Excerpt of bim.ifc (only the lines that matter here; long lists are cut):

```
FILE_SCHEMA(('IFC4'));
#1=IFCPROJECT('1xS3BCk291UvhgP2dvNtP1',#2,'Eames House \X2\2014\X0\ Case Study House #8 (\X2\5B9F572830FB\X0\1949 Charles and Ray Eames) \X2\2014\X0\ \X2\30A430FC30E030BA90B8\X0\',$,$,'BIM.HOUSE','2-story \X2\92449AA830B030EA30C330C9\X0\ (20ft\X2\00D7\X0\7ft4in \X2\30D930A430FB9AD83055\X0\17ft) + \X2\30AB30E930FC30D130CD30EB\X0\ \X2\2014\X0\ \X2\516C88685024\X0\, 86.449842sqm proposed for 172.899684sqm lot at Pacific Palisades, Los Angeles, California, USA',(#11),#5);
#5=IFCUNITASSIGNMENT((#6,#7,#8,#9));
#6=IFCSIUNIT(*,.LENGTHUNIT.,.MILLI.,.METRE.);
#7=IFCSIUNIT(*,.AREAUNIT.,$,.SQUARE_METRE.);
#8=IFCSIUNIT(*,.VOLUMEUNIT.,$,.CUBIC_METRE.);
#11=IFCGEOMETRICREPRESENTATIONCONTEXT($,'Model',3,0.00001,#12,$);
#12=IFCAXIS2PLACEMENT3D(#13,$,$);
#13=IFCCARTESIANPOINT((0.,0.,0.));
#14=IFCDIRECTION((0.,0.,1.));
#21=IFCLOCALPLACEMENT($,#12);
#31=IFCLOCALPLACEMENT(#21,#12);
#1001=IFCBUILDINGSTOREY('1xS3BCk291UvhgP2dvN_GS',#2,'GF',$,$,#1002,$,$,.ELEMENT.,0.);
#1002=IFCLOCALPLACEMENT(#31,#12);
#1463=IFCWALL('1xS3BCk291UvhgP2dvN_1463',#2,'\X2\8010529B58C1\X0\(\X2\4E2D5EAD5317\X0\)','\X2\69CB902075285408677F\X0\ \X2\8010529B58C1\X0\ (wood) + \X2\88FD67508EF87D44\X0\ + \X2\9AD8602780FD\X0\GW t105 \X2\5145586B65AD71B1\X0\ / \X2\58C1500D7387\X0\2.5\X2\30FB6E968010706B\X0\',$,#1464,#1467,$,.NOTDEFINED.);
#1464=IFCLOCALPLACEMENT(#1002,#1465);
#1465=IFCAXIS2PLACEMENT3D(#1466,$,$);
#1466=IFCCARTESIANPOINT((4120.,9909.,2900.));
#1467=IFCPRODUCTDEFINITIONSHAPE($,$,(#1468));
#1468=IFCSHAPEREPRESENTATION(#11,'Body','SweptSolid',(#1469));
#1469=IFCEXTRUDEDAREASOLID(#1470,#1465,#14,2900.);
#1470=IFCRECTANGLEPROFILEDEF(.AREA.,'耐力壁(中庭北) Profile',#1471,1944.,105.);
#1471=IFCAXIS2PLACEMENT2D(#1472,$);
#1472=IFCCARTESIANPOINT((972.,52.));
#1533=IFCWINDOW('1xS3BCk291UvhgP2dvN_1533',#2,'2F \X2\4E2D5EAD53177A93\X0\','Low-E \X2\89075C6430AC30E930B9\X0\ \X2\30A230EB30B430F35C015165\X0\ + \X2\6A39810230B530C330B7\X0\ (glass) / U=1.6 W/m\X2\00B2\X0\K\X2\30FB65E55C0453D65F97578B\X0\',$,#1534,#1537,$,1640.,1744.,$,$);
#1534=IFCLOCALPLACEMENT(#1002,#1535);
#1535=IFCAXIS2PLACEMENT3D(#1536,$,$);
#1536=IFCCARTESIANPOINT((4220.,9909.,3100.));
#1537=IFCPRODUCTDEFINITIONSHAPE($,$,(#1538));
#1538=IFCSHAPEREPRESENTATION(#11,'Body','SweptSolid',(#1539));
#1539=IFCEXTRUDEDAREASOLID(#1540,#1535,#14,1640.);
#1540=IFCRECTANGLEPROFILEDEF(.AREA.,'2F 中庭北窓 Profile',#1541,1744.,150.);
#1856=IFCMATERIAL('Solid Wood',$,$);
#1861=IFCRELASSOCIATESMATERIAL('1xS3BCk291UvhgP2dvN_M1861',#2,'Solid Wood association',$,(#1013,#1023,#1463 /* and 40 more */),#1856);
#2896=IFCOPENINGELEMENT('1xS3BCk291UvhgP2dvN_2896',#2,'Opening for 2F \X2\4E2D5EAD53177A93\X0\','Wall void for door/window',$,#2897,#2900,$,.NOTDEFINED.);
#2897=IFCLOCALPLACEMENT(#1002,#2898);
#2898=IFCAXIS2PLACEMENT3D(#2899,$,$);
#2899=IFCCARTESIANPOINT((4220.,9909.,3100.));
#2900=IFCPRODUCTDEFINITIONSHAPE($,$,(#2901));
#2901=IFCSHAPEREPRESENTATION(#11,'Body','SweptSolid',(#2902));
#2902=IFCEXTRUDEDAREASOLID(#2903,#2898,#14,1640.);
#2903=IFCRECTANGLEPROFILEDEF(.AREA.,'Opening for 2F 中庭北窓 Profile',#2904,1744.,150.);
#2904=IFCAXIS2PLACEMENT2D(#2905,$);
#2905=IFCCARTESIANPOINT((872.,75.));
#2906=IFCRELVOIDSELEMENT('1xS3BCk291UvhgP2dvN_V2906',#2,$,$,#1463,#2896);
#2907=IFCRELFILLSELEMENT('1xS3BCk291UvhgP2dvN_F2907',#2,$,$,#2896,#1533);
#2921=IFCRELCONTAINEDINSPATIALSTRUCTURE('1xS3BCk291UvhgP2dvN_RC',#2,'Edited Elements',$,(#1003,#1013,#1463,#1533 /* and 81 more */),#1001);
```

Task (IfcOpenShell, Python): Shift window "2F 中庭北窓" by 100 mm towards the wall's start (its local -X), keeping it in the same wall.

```python
import ifcopenshell
import ifcopenshell.api.geometry
import ifcopenshell.util.placement

model = ifcopenshell.open("bim.ifc")

window = model.by_guid("1xS3BCk291UvhgP2dvN_1533")
opening = window.FillsVoids[0].RelatingOpeningElement
wall = opening.VoidsElements[0].RelatingBuildingElement

wall_matrix = ifcopenshell.util.placement.get_local_placement(wall.ObjectPlacement)
shift = wall_matrix[:3, 0] * -100.0
before = ifcopenshell.util.placement.get_local_placement(window.ObjectPlacement)[:3, 3].copy()

# The window is not placed relative to its opening, so move both.
for product in (opening, window):
    matrix = ifcopenshell.util.placement.get_local_placement(product.ObjectPlacement)
    matrix[:3, 3] += shift
    ifcopenshell.api.geometry.edit_object_placement(model, product=product, matrix=matrix, is_si=False)

after = ifcopenshell.util.placement.get_local_placement(window.ObjectPlacement)[:3, 3]
print("window moved by", (after - before).round(3) + 0.0)

model.write("bim_updated.ifc")
```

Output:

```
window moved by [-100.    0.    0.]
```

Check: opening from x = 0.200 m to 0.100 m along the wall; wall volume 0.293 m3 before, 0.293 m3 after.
